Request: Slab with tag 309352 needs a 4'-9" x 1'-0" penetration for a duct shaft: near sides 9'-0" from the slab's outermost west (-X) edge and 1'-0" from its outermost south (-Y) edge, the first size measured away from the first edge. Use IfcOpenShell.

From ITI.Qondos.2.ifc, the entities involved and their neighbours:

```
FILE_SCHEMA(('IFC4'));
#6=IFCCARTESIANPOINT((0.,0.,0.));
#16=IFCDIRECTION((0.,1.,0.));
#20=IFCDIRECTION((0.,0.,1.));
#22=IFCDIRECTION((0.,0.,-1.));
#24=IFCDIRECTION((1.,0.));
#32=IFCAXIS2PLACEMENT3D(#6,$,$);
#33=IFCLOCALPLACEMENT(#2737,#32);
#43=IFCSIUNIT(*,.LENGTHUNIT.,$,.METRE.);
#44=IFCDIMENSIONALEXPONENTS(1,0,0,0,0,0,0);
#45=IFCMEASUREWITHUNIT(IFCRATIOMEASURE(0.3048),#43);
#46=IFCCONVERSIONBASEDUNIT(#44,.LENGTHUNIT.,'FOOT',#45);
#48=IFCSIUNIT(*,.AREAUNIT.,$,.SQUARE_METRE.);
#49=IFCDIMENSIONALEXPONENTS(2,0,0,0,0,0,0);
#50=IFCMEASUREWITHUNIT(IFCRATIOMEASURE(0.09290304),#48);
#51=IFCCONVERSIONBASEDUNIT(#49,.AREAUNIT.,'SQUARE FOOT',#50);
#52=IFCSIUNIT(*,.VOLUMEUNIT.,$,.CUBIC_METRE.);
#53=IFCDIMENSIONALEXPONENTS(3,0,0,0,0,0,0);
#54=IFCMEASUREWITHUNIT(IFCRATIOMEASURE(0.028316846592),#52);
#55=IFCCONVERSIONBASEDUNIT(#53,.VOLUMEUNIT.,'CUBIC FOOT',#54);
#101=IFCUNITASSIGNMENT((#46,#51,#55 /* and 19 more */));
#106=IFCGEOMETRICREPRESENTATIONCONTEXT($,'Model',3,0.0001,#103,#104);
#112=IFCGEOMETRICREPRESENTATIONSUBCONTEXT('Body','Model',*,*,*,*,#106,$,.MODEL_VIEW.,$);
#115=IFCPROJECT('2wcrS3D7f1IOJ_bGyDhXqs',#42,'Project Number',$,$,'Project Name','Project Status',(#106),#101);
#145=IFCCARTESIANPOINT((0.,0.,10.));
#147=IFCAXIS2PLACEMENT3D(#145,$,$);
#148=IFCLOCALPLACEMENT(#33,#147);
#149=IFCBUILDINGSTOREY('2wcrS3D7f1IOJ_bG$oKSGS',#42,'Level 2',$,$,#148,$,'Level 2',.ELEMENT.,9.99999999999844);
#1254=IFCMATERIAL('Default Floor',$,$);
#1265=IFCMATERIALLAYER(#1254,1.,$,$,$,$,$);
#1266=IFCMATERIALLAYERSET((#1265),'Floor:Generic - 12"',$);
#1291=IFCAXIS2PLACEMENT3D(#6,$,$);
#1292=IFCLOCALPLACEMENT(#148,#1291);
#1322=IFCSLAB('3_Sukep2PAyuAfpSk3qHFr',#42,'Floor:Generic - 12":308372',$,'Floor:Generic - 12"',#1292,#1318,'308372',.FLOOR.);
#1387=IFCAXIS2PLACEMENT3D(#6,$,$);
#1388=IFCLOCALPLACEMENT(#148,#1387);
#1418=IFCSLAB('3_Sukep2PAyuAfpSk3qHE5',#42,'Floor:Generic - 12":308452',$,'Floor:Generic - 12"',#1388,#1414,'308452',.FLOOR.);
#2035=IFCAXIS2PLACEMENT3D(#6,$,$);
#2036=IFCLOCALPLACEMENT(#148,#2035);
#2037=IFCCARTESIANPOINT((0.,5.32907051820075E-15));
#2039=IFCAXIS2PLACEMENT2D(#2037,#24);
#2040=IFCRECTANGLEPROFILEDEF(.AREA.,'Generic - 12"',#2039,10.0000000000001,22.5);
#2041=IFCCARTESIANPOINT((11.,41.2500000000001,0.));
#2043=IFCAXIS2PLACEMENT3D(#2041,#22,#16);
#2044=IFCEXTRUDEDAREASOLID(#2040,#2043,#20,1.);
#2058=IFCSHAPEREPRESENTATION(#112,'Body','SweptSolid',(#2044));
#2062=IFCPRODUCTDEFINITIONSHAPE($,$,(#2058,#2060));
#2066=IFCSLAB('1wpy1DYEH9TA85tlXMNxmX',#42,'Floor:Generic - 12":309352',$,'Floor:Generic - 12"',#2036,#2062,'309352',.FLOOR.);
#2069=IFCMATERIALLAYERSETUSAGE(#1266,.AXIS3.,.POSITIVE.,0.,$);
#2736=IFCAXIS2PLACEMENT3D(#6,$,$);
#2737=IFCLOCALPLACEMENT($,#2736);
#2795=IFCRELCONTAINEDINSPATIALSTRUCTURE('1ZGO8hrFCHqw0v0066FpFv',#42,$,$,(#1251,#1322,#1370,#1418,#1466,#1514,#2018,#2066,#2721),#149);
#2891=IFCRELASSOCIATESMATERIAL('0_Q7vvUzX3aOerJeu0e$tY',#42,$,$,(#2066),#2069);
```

```python
import numpy as np
import ifcopenshell
import ifcopenshell.api.feature
import ifcopenshell.api.geometry
import ifcopenshell.api.root
import ifcopenshell.geom
import ifcopenshell.util.placement
import ifcopenshell.util.representation
import ifcopenshell.util.shape
import ifcopenshell.util.unit

model = ifcopenshell.open("ITI.Qondos.2.ifc")
unit_scale = ifcopenshell.util.unit.calculate_unit_scale(model)
settings = ifcopenshell.geom.settings()


def volume(element):
    """Net volume in cubic metres, openings subtracted."""
    shape = ifcopenshell.geom.create_shape(settings, element)
    return ifcopenshell.util.shape.get_volume(shape.geometry)


slab = model.by_guid("1wpy1DYEH9TA85tlXMNxmX")
before = volume(slab)

# Extent in the slab's own axes, in metres. The edges named are its -X and -Y sides.
slab_shape = ifcopenshell.geom.create_shape(settings, slab)
vertices = ifcopenshell.util.shape.get_vertices(slab_shape.geometry)
x_min, y_min, bottom = vertices.min(axis=0)
top = vertices[:, 2].max()

opening = ifcopenshell.api.root.create_entity(model, ifc_class="IfcOpeningElement", name="Duct shaft opening", predefined_type="OPENING")
context = ifcopenshell.util.representation.get_context(model, "Model", "Body", "MODEL_VIEW")
width, depth = 1.4478, 0.3048
outline = [(0.0, 0.0), (width, 0.0), (width, depth), (0.0, depth), (0.0, 0.0)]
# Overshoot both faces by 50 mm so the cut is clean.
shape = ifcopenshell.api.geometry.add_slab_representation(
    model, context=context, depth=top - bottom + 0.1, polyline=outline
)
ifcopenshell.api.geometry.assign_representation(model, product=opening, representation=shape)

matrix = ifcopenshell.util.placement.get_local_placement(slab.ObjectPlacement)
matrix[:, 3] = matrix @ np.append(np.array([x_min + 2.7432, y_min + 0.3048, bottom - 0.05]) / unit_scale, 1.0)
ifcopenshell.api.geometry.edit_object_placement(model, product=opening, matrix=matrix, is_si=False)
ifcopenshell.api.feature.add_feature(model, feature=opening, element=slab)

after = volume(slab)

print(f"slab volume {before:.3f} -> {after:.3f} m3")

model.write("ITI.Qondos.2_v2.ifc")
```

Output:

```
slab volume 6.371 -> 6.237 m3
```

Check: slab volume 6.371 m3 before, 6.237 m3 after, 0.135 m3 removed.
